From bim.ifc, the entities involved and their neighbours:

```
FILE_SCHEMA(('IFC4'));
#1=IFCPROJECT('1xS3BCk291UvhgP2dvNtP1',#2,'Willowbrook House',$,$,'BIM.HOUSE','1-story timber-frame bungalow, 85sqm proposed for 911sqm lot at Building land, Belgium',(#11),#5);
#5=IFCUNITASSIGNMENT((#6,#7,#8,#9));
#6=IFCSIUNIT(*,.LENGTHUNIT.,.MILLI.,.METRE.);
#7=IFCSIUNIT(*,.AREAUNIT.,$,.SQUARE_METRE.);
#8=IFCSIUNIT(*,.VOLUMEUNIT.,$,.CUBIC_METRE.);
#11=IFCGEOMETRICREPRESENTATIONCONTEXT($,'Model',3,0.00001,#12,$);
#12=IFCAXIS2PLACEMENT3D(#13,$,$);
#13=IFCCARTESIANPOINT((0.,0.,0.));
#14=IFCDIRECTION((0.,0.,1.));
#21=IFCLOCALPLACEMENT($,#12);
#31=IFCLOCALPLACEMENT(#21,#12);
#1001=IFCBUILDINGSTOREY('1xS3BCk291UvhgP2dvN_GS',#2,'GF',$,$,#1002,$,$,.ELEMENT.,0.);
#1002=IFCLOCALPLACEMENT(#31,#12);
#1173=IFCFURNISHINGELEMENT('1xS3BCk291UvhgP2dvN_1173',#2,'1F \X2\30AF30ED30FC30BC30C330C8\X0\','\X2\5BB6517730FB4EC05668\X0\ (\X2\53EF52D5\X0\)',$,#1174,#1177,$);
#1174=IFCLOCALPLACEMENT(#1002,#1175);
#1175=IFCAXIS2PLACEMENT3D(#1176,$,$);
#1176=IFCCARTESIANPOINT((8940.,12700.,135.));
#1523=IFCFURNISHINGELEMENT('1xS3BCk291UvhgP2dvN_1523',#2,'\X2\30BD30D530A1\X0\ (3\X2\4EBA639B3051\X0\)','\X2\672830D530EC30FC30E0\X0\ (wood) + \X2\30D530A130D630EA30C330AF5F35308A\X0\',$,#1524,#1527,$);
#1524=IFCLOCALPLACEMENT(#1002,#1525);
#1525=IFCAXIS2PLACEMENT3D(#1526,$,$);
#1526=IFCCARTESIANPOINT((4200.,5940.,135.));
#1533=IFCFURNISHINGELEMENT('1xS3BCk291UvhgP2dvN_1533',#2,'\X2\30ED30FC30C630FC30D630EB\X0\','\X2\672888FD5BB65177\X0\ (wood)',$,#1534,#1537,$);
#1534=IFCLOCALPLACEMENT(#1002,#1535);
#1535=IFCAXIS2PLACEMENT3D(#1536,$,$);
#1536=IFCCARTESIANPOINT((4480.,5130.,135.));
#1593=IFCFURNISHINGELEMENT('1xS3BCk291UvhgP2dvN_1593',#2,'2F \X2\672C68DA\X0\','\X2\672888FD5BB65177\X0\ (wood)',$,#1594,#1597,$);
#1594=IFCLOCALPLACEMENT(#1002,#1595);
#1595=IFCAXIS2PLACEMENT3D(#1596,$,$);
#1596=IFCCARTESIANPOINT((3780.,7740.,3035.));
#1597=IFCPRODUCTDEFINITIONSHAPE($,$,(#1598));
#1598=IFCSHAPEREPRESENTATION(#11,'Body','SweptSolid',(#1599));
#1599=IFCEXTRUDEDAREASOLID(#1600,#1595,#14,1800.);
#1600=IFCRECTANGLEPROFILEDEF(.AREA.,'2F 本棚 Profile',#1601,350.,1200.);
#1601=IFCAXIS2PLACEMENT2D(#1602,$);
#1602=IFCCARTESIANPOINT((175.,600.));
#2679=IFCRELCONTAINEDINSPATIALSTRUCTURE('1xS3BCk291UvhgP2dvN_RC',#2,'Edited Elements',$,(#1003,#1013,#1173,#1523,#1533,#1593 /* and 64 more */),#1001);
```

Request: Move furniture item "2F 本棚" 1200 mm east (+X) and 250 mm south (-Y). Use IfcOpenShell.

```python
import ifcopenshell
import ifcopenshell.api.geometry
import ifcopenshell.util.placement

model = ifcopenshell.open("bim.ifc")

item = model.by_id(1593)
matrix = ifcopenshell.util.placement.get_local_placement(item.ObjectPlacement)
matrix[0, 3] += 1200.0
matrix[1, 3] -= 250.0
ifcopenshell.api.geometry.edit_object_placement(model, product=item, matrix=matrix, is_si=False)

print(ifcopenshell.util.placement.get_local_placement(item.ObjectPlacement).round(3) + 0.0)

model.write("bim_updated.ifc")
```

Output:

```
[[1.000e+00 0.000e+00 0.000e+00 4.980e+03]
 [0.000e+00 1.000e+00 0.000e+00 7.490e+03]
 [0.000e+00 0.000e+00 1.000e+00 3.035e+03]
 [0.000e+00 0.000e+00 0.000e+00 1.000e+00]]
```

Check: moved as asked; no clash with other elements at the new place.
